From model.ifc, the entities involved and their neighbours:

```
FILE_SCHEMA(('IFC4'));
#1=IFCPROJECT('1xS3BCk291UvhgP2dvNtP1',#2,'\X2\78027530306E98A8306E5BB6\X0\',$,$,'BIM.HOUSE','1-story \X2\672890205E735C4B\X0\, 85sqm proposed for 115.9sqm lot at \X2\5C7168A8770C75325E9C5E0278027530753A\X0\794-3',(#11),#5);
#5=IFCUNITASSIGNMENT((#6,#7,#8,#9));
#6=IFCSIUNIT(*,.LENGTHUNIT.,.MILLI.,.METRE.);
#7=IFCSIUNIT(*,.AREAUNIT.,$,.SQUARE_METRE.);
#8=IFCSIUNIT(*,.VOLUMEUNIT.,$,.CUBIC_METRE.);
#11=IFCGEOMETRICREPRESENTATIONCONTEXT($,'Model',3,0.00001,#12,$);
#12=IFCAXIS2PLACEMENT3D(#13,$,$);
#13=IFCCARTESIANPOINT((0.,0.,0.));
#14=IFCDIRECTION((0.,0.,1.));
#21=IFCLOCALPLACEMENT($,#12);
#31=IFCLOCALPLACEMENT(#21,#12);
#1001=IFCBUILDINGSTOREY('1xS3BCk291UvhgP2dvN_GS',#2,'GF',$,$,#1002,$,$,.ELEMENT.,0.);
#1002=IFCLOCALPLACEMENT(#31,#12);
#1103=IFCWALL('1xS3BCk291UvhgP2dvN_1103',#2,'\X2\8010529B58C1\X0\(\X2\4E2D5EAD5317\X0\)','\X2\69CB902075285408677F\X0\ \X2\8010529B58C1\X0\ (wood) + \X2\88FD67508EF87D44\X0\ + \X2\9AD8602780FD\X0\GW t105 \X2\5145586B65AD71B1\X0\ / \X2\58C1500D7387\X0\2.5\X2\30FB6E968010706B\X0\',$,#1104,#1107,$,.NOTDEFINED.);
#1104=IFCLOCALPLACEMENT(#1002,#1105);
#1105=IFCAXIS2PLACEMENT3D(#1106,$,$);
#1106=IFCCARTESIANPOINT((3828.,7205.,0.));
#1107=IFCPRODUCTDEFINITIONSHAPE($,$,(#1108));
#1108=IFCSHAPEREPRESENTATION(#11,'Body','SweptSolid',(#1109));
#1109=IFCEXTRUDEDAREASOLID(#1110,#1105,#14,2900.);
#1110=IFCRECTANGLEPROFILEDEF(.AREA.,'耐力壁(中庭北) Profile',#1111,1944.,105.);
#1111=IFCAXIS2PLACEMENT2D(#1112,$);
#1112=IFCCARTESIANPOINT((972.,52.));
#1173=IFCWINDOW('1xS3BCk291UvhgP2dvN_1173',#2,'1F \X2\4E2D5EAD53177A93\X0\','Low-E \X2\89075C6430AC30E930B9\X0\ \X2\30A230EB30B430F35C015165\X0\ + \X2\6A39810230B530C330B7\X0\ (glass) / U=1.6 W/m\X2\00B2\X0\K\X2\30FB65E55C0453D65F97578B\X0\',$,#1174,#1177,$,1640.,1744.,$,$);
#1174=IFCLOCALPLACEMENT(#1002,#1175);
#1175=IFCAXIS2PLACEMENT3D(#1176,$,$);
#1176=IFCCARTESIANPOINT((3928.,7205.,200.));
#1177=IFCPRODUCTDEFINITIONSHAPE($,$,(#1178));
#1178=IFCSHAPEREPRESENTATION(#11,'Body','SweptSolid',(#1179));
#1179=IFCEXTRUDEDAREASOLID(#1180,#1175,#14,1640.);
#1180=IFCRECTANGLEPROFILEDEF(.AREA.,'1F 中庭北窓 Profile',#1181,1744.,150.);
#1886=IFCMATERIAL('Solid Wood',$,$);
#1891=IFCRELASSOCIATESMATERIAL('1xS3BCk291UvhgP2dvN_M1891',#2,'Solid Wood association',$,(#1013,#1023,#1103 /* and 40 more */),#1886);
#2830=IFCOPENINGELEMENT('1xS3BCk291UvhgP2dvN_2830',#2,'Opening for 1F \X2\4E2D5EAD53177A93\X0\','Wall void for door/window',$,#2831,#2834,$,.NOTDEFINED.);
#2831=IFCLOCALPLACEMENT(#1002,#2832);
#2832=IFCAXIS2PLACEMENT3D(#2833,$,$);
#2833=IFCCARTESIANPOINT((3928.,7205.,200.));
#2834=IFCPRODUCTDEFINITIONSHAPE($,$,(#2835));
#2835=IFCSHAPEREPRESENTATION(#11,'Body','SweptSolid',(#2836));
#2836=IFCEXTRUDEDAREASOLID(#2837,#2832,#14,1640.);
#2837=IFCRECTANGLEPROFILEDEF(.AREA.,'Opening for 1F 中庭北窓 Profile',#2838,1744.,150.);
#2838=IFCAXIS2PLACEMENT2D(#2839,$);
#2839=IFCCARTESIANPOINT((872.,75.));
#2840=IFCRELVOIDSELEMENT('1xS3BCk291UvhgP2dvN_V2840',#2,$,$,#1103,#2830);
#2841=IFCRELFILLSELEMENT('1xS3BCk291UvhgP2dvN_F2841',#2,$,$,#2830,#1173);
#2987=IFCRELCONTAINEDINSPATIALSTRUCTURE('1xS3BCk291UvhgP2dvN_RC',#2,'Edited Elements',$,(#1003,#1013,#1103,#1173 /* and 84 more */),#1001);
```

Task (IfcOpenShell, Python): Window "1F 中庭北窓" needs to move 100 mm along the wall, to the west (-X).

```python
import ifcopenshell
import ifcopenshell.api.geometry
import ifcopenshell.util.placement
import ifcopenshell.util.unit

model = ifcopenshell.open("model.ifc")
unit_scale = ifcopenshell.util.unit.calculate_unit_scale(model)

window = model.by_id(1173)
opening = window.FillsVoids[0].RelatingOpeningElement
wall = opening.VoidsElements[0].RelatingBuildingElement

wall_matrix = ifcopenshell.util.placement.get_local_placement(wall.ObjectPlacement)
shift = wall_matrix[:3, 0] * -0.1 / unit_scale
before = ifcopenshell.util.placement.get_local_placement(window.ObjectPlacement)[:3, 3].copy()

# The window is not placed relative to its opening, so move both.
for product in (opening, window):
    matrix = ifcopenshell.util.placement.get_local_placement(product.ObjectPlacement)
    matrix[:3, 3] += shift
    ifcopenshell.api.geometry.edit_object_placement(model, product=product, matrix=matrix, is_si=False)

after = ifcopenshell.util.placement.get_local_placement(window.ObjectPlacement)[:3, 3]
print("window moved by", (after - before).round(3) + 0.0)

model.write("model_edited.ifc")
```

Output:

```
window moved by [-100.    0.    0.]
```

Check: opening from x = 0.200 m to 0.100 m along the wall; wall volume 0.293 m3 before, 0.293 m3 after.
